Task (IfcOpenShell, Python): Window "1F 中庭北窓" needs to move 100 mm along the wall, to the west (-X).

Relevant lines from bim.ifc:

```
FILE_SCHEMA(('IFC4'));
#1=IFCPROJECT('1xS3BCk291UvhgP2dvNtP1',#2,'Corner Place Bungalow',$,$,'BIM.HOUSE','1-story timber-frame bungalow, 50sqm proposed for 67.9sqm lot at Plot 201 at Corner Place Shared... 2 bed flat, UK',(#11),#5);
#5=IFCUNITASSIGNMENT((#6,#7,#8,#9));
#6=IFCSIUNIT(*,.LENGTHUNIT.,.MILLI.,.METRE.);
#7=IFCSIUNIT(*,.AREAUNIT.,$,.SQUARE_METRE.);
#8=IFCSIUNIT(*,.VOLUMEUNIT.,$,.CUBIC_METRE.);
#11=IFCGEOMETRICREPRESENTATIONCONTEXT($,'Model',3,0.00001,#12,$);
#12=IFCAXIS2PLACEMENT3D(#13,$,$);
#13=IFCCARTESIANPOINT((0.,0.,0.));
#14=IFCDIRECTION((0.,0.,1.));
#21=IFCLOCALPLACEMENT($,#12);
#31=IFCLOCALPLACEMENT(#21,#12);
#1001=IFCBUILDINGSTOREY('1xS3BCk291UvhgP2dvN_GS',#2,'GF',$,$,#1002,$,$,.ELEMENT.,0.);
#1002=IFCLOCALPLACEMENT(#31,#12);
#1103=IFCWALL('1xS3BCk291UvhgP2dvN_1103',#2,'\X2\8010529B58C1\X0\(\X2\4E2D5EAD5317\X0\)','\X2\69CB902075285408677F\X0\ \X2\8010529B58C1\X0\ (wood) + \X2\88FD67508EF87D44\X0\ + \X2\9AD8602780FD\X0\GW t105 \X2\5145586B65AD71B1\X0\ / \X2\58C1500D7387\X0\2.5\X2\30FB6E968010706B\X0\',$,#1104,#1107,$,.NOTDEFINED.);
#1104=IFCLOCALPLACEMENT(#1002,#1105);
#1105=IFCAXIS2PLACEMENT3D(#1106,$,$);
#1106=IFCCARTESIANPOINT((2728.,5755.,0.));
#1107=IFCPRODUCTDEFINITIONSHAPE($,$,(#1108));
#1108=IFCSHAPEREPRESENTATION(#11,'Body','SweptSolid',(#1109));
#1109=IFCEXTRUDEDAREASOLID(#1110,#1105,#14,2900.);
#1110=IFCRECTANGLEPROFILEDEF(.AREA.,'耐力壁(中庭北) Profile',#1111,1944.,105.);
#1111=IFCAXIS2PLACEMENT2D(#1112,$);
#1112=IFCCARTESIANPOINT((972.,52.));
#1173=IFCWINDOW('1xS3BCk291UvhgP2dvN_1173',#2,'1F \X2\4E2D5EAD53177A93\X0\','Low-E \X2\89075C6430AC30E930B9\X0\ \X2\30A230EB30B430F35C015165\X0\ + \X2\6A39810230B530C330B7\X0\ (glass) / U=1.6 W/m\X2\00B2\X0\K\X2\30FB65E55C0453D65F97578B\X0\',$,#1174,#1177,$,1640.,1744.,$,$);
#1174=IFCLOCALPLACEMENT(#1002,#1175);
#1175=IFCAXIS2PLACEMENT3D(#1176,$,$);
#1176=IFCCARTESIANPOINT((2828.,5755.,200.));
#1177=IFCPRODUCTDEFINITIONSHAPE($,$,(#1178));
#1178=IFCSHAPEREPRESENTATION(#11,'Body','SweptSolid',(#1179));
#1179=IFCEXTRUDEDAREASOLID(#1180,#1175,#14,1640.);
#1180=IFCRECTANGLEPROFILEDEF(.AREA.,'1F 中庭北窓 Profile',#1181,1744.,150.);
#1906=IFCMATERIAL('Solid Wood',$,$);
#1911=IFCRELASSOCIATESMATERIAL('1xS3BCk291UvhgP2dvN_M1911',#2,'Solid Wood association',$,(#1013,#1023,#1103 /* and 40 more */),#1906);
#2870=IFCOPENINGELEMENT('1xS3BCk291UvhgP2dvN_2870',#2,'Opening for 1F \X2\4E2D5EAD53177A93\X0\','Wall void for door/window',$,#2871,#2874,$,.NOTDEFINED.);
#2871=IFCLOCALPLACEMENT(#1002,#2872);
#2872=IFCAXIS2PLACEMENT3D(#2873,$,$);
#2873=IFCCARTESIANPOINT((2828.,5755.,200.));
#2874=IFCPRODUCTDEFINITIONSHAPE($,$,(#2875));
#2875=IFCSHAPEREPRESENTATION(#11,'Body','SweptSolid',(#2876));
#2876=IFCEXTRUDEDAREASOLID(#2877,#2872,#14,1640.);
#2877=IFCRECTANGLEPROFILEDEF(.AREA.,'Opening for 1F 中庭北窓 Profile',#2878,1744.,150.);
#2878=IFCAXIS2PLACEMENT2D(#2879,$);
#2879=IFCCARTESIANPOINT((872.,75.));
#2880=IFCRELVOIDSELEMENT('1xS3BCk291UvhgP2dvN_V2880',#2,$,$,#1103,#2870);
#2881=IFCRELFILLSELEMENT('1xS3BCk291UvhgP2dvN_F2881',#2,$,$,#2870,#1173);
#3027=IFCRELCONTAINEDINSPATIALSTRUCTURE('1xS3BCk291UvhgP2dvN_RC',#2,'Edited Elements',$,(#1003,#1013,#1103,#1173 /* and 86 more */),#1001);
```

```python
import ifcopenshell
import ifcopenshell.api.geometry
import ifcopenshell.util.placement
import ifcopenshell.util.unit

model = ifcopenshell.open("bim.ifc")
unit_scale = ifcopenshell.util.unit.calculate_unit_scale(model)

window = model.by_guid("1xS3BCk291UvhgP2dvN_1173")
opening = window.FillsVoids[0].RelatingOpeningElement
wall = opening.VoidsElements[0].RelatingBuildingElement

wall_matrix = ifcopenshell.util.placement.get_local_placement(wall.ObjectPlacement)
shift = wall_matrix[:3, 0] * -0.1 / unit_scale
before = ifcopenshell.util.placement.get_local_placement(window.ObjectPlacement)[:3, 3].copy()

# The window is not placed relative to its opening, so move both.
for product in (opening, window):
    matrix = ifcopenshell.util.placement.get_local_placement(product.ObjectPlacement)
    matrix[:3, 3] += shift
    ifcopenshell.api.geometry.edit_object_placement(model, product=product, matrix=matrix, is_si=False)

after = ifcopenshell.util.placement.get_local_placement(window.ObjectPlacement)[:3, 3]
print("window moved by", (after - before).round(3) + 0.0)

model.write("bim-out.ifc")
```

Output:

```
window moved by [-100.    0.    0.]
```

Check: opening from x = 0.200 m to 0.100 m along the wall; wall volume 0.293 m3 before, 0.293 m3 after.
